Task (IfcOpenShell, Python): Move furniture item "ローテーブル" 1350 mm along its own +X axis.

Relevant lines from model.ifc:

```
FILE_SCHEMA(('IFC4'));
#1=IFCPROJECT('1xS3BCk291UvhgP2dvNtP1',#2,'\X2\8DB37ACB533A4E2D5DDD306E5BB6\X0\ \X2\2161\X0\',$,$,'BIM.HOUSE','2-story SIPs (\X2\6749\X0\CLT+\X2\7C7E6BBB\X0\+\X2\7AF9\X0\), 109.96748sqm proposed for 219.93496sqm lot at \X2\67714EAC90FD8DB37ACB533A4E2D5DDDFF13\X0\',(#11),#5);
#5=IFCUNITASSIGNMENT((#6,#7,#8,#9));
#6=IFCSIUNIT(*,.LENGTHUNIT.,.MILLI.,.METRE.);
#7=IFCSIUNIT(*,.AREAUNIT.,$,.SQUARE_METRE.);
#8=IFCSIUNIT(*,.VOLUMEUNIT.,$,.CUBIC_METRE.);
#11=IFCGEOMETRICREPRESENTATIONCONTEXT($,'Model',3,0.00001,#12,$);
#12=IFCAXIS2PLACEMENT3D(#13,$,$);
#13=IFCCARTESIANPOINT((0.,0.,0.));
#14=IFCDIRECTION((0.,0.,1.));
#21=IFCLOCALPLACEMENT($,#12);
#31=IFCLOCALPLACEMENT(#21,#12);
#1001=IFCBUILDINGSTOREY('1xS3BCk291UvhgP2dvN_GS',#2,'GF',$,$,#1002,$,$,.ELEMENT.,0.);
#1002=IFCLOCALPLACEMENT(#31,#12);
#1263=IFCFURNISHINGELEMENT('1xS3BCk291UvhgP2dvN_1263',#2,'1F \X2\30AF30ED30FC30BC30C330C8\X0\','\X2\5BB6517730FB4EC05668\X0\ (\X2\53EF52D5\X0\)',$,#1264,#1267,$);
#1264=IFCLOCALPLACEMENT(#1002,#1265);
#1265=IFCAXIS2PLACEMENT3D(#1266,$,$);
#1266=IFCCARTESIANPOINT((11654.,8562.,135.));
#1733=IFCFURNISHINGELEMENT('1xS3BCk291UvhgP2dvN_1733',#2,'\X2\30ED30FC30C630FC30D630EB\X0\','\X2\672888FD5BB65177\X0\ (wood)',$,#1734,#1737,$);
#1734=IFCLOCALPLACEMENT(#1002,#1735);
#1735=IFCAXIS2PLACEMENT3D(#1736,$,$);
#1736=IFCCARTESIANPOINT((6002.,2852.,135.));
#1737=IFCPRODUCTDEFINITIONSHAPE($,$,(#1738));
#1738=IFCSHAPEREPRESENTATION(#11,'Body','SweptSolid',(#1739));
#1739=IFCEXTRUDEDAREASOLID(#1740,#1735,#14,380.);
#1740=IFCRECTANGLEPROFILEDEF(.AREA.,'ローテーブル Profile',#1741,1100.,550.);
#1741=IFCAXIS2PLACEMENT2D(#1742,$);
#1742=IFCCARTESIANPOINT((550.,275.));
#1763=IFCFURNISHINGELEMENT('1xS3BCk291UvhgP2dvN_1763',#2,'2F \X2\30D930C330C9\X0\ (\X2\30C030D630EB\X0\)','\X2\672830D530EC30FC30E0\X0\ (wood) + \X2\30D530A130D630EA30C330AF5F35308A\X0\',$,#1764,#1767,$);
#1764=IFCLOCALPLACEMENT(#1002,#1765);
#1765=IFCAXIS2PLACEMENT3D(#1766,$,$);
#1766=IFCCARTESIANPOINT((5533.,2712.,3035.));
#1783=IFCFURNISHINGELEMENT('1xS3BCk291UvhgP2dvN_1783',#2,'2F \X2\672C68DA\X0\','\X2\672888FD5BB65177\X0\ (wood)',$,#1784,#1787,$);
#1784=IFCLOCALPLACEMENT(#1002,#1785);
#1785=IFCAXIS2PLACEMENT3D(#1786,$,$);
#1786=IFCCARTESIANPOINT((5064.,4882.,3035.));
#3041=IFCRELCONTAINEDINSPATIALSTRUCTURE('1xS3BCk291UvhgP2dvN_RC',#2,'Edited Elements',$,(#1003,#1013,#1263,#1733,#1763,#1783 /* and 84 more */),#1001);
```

```python
import ifcopenshell
import ifcopenshell.api.geometry
import ifcopenshell.util.placement
import ifcopenshell.util.unit

model = ifcopenshell.open("model.ifc")
unit_scale = ifcopenshell.util.unit.calculate_unit_scale(model)

item = model.by_guid("1xS3BCk291UvhgP2dvN_1733")
matrix = ifcopenshell.util.placement.get_local_placement(item.ObjectPlacement)
matrix[:3, 3] += matrix[:3, 0] * 1.35 / unit_scale
ifcopenshell.api.geometry.edit_object_placement(model, product=item, matrix=matrix, is_si=False)

print(ifcopenshell.util.placement.get_local_placement(item.ObjectPlacement).round(3) + 0.0)

model.write("model_v2.ifc")
```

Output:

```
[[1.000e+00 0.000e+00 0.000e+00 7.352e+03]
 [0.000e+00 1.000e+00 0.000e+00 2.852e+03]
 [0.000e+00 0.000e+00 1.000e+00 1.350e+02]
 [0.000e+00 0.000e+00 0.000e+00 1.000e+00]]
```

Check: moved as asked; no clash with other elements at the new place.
